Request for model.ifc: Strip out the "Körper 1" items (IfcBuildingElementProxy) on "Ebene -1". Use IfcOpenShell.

First a look at what the model holds.

```python
import ifcopenshell
import ifcopenshell.util.element

model = ifcopenshell.open("model.ifc")
print(model.schema)
storey = next(s for s in model.by_type("IfcBuildingStorey") if s.Name == "Ebene -1")
proxies = [e for e in ifcopenshell.util.element.get_decomposition(storey) if e.is_a("IfcBuildingElementProxy")]
seen = {}
for e in proxies:
    element_type = ifcopenshell.util.element.get_type(e)
    name = element_type.Name if element_type not in (None, e) else None
    seen[name] = seen.get(name, 0) + 1
for name, count in sorted(seen.items(), key=str):
    print(count, "x", name)
```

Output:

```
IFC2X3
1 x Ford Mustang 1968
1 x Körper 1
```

```python
import ifcopenshell
import ifcopenshell.api.root
import ifcopenshell.util.element

model = ifcopenshell.open("model.ifc")

storey = next(s for s in model.by_type("IfcBuildingStorey") if s.Name == "Ebene -1")
proxies = [e for e in ifcopenshell.util.element.get_decomposition(storey) if e.is_a("IfcBuildingElementProxy")]
targets = [e for e in proxies if (t := ifcopenshell.util.element.get_type(e)) not in (None, e) and t.Name == "Körper 1"]

for e in targets:
    ifcopenshell.api.root.remove_product(model, product=e)
print(len(targets), "removed")

model.write("model_updated.ifc")
```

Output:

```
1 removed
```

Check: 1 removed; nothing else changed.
